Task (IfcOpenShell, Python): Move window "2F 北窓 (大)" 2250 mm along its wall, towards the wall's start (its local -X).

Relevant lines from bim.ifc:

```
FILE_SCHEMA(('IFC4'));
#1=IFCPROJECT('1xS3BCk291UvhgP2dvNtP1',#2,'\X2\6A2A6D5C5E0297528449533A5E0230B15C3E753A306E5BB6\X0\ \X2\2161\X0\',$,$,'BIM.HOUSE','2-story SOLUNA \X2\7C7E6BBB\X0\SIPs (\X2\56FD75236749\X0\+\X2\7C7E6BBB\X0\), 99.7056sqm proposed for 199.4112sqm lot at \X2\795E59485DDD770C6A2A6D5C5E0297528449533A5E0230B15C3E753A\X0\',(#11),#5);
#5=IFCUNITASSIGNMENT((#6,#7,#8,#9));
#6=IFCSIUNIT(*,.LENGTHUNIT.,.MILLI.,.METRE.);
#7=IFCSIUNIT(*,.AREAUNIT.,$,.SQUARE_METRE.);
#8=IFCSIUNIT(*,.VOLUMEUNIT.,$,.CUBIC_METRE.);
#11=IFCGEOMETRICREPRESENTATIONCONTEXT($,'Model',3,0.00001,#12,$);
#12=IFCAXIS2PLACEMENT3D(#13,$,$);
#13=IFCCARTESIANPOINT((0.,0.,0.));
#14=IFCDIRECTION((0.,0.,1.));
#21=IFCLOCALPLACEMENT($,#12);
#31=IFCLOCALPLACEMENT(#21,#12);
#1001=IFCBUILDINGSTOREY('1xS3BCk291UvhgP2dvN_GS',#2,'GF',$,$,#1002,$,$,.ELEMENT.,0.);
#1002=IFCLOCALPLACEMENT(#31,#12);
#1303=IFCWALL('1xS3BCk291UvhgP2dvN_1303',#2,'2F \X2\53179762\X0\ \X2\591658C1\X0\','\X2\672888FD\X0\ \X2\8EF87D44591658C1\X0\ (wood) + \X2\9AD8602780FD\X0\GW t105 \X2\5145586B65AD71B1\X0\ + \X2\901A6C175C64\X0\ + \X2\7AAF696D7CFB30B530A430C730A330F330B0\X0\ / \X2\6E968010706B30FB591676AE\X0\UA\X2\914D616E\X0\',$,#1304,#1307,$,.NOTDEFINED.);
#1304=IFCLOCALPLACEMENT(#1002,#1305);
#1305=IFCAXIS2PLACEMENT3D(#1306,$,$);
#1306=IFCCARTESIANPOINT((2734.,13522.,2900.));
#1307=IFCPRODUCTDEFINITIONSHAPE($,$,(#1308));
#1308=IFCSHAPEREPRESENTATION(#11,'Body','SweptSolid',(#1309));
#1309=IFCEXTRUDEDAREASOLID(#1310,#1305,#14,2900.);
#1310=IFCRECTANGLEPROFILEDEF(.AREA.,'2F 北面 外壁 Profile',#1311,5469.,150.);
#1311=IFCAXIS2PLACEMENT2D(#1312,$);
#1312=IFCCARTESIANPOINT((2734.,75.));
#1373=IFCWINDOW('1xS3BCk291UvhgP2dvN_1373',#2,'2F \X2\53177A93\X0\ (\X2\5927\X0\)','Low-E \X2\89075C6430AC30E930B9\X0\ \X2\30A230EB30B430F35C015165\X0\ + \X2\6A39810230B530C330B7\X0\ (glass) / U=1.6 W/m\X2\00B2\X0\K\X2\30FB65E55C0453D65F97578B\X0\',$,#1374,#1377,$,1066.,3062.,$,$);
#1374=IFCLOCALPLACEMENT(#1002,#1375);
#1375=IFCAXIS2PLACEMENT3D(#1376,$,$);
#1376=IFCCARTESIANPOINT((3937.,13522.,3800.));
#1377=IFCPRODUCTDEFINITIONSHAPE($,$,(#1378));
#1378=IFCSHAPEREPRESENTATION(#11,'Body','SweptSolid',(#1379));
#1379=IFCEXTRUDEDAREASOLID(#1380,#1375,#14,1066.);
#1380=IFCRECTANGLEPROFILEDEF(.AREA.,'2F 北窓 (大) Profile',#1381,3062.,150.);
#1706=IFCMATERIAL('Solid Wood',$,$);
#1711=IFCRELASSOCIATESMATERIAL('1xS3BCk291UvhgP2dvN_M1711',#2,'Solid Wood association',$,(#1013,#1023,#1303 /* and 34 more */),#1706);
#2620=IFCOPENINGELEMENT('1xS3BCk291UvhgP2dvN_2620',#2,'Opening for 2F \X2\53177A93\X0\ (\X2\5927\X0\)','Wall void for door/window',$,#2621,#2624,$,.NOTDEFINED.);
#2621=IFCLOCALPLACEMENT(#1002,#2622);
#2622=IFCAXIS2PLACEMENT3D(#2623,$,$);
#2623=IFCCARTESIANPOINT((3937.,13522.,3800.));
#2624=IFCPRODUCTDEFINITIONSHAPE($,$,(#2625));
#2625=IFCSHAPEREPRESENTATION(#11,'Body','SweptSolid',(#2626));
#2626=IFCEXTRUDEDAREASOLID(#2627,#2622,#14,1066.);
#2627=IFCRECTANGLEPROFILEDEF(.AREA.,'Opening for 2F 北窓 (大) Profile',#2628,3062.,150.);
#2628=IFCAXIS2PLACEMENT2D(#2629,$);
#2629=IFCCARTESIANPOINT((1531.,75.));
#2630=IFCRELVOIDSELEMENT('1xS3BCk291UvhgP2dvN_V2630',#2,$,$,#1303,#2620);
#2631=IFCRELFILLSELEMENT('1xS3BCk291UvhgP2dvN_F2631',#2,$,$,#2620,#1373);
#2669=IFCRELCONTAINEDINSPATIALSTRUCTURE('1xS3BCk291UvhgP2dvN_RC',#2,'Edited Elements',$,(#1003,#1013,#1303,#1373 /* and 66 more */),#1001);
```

```python
import ifcopenshell
import ifcopenshell.api.geometry
import ifcopenshell.util.placement
import ifcopenshell.util.unit

model = ifcopenshell.open("bim.ifc")
unit_scale = ifcopenshell.util.unit.calculate_unit_scale(model)

window = model.by_id(1373)
opening = window.FillsVoids[0].RelatingOpeningElement
wall = opening.VoidsElements[0].RelatingBuildingElement

wall_matrix = ifcopenshell.util.placement.get_local_placement(wall.ObjectPlacement)
shift = wall_matrix[:3, 0] * -2.25 / unit_scale
before = ifcopenshell.util.placement.get_local_placement(window.ObjectPlacement)[:3, 3].copy()

# The window is not placed relative to its opening, so move both.
for product in (opening, window):
    matrix = ifcopenshell.util.placement.get_local_placement(product.ObjectPlacement)
    matrix[:3, 3] += shift
    ifcopenshell.api.geometry.edit_object_placement(model, product=product, matrix=matrix, is_si=False)

after = ifcopenshell.util.placement.get_local_placement(window.ObjectPlacement)[:3, 3]
print("window moved by", (after - before).round(3) + 0.0)

model.write("bim_edited.ifc")
```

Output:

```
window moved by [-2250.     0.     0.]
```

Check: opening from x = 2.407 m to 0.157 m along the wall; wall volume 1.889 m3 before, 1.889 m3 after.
